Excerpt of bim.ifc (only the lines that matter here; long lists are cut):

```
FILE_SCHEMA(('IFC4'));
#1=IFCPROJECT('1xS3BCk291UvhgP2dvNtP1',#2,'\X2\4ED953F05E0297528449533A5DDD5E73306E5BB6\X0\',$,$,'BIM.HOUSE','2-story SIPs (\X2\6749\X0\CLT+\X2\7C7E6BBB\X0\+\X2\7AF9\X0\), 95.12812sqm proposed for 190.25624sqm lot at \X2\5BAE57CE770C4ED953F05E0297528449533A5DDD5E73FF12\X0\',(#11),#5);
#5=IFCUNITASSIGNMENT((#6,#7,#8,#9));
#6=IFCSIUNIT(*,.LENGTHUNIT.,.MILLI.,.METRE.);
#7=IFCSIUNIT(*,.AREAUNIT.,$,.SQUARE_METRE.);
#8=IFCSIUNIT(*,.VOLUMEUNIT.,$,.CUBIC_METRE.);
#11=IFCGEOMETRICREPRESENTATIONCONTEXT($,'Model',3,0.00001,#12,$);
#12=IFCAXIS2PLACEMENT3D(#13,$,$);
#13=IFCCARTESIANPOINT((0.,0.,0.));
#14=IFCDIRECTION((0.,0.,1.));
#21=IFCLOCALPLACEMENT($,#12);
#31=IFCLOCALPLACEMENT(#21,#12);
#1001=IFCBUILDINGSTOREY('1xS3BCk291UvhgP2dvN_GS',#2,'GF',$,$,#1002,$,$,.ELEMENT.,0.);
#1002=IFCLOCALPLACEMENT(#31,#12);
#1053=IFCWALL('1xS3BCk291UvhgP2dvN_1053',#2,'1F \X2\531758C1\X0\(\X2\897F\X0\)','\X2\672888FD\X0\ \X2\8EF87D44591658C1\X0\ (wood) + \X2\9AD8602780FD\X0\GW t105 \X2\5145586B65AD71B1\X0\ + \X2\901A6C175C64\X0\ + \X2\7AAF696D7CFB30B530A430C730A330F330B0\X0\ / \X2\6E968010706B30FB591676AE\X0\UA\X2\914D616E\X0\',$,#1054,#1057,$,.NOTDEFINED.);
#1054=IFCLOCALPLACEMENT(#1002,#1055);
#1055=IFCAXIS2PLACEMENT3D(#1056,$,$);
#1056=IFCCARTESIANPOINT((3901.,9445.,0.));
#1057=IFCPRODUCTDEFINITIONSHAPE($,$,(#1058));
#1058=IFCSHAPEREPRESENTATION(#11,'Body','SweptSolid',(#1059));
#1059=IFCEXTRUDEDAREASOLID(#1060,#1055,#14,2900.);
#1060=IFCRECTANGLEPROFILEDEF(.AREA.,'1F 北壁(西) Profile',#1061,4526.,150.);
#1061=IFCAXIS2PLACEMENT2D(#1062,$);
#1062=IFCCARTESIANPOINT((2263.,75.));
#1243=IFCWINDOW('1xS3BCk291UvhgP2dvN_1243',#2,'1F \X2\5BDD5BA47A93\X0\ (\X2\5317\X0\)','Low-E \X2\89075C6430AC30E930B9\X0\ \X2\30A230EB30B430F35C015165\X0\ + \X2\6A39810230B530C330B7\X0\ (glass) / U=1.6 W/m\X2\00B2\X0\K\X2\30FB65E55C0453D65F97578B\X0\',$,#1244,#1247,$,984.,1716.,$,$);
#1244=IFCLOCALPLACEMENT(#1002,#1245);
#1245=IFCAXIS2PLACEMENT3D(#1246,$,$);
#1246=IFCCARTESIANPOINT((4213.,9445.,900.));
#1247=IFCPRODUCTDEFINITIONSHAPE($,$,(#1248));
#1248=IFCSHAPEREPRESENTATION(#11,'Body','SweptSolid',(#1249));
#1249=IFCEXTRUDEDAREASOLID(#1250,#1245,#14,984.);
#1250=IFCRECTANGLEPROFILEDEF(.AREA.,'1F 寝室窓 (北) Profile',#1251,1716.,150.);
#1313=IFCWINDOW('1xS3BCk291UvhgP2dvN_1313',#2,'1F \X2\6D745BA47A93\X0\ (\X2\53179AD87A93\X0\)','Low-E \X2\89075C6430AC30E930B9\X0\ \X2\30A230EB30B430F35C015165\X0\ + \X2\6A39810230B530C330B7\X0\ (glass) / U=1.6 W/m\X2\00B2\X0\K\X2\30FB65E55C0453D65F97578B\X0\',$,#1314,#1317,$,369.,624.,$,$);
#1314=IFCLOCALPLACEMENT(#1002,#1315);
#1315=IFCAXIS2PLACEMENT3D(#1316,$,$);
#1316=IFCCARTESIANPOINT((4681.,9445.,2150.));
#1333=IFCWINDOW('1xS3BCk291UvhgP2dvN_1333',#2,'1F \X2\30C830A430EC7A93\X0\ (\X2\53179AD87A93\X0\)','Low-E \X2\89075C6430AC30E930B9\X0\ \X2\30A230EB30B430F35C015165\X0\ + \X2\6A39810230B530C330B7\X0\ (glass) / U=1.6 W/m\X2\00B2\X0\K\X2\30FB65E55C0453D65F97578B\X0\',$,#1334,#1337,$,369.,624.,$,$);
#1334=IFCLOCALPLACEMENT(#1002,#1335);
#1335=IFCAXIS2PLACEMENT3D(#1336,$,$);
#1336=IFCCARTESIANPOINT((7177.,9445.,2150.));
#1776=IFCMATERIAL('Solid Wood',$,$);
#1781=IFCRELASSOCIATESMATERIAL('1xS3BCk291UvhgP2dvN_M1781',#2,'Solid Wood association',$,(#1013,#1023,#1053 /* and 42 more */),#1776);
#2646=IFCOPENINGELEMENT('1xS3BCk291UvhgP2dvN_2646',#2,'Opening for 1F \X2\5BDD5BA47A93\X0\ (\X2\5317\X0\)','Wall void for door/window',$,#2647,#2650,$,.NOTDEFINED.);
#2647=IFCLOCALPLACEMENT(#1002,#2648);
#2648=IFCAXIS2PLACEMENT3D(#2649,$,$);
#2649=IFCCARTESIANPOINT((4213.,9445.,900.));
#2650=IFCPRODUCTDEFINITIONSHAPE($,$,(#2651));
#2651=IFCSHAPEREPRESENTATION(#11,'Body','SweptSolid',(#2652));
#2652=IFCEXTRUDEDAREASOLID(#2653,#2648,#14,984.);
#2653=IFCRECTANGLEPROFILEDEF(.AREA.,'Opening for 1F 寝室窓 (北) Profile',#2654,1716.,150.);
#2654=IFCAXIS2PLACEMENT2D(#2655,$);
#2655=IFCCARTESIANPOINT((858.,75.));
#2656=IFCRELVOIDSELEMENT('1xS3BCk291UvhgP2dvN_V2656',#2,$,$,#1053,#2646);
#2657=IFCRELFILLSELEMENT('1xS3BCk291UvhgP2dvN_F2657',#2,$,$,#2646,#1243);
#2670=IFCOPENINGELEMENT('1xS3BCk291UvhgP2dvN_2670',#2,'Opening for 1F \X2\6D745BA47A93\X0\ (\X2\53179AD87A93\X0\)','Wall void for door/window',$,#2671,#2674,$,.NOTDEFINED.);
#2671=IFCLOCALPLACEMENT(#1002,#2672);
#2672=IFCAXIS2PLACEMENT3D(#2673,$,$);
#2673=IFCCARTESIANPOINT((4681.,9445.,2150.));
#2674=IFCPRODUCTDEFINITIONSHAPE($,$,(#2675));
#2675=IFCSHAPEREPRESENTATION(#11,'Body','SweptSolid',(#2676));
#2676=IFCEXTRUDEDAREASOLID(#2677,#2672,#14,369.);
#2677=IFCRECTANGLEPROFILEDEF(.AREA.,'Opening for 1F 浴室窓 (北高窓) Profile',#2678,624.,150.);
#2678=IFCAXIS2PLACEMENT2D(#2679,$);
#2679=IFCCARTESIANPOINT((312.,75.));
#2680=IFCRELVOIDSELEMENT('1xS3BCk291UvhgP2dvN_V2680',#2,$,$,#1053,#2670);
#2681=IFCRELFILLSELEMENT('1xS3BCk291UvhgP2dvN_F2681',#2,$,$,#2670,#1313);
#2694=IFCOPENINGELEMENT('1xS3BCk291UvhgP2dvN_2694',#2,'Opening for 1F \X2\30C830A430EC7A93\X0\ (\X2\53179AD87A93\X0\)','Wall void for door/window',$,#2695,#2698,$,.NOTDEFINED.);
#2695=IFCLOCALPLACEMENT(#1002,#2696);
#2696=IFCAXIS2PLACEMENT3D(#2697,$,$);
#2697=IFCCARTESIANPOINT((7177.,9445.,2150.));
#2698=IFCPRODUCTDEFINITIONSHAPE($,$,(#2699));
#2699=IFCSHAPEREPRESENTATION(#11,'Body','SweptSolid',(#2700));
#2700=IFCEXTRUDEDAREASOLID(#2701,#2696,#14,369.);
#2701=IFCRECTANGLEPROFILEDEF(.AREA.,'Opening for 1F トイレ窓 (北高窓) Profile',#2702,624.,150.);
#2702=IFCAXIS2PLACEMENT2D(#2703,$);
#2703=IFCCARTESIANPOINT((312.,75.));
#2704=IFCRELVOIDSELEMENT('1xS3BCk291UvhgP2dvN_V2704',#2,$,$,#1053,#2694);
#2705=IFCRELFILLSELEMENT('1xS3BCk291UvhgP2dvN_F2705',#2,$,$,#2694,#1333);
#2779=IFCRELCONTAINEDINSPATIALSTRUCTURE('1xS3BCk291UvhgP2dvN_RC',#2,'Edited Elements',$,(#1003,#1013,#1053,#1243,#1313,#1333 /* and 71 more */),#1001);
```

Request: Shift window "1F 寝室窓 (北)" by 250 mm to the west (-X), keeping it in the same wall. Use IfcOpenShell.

```python
import ifcopenshell
import ifcopenshell.api.geometry
import ifcopenshell.util.placement
import ifcopenshell.util.unit

model = ifcopenshell.open("bim.ifc")
unit_scale = ifcopenshell.util.unit.calculate_unit_scale(model)

window = model.by_id(1243)
opening = window.FillsVoids[0].RelatingOpeningElement
wall = opening.VoidsElements[0].RelatingBuildingElement

wall_matrix = ifcopenshell.util.placement.get_local_placement(wall.ObjectPlacement)
shift = wall_matrix[:3, 0] * -0.25 / unit_scale
before = ifcopenshell.util.placement.get_local_placement(window.ObjectPlacement)[:3, 3].copy()

# The window is not placed relative to its opening, so move both.
for product in (opening, window):
    matrix = ifcopenshell.util.placement.get_local_placement(product.ObjectPlacement)
    matrix[:3, 3] += shift
    ifcopenshell.api.geometry.edit_object_placement(model, product=product, matrix=matrix, is_si=False)

after = ifcopenshell.util.placement.get_local_placement(window.ObjectPlacement)[:3, 3]
print("window moved by", (after - before).round(3) + 0.0)

model.write("bim_rev.ifc")
```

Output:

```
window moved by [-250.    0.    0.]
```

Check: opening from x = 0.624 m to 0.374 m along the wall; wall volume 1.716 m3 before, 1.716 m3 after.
